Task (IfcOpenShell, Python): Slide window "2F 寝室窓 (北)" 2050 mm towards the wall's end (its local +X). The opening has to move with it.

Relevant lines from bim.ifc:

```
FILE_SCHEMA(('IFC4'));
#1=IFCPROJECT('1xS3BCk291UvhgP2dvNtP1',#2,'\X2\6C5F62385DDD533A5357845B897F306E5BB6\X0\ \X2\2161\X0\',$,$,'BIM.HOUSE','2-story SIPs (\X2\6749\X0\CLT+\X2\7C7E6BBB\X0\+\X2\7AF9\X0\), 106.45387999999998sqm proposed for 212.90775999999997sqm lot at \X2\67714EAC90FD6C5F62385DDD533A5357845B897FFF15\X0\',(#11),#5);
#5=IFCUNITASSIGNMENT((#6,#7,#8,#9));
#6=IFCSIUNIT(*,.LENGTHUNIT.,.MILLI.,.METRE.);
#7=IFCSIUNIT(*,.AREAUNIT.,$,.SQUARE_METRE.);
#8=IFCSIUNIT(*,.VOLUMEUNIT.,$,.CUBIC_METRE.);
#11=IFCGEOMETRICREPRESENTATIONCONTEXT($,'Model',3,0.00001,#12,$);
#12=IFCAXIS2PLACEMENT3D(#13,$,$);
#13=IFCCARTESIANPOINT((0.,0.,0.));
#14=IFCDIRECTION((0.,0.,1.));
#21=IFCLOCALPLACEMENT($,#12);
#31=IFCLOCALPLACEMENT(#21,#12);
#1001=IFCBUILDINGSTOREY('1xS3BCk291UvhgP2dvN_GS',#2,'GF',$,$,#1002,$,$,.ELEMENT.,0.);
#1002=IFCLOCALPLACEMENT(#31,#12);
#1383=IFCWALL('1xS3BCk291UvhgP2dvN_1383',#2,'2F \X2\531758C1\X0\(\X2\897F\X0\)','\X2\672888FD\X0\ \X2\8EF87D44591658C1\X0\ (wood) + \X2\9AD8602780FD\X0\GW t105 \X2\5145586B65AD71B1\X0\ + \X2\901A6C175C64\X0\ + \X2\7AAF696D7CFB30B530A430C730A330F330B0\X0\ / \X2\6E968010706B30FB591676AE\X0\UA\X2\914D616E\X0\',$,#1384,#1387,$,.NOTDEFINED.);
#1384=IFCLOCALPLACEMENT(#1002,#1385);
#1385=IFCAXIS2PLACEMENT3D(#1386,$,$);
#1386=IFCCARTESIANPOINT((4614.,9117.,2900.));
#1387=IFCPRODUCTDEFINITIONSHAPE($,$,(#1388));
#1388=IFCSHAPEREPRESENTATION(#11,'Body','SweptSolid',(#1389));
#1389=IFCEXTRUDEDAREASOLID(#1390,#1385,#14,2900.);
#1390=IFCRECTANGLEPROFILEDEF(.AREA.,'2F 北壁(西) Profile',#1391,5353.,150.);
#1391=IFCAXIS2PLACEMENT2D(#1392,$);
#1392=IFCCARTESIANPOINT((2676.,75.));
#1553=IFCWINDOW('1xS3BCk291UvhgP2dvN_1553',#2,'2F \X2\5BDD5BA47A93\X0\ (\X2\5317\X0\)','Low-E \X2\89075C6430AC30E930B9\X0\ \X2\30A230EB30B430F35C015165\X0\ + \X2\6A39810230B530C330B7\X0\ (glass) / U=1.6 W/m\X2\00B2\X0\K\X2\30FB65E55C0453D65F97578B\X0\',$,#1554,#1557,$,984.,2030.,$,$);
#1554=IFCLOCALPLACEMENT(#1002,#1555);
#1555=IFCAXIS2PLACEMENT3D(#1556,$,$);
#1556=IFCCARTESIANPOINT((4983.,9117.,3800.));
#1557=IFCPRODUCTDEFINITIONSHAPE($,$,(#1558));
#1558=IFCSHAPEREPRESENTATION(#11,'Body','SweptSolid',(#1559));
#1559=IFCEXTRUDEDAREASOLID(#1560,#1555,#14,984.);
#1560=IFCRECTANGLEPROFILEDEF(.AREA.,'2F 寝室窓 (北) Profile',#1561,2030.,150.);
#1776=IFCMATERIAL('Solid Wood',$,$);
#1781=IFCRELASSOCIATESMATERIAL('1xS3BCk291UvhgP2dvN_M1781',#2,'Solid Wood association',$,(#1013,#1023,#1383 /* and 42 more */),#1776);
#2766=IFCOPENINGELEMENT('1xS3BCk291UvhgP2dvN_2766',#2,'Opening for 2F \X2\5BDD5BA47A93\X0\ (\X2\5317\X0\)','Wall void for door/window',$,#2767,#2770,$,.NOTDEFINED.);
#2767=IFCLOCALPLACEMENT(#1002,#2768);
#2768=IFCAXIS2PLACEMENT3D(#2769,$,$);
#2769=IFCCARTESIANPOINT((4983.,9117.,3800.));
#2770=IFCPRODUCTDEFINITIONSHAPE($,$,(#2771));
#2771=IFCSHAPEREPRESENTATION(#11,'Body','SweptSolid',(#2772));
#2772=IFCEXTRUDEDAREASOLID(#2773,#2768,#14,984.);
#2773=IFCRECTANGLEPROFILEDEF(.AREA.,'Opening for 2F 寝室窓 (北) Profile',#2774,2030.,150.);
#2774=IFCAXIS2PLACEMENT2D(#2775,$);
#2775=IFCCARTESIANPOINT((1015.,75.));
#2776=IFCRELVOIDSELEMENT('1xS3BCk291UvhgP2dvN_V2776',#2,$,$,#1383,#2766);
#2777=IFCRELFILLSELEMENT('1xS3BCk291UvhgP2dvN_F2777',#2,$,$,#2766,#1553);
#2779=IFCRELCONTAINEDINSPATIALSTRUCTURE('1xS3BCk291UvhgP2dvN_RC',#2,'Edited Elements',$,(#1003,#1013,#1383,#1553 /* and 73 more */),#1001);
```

```python
import ifcopenshell
import ifcopenshell.api.geometry
import ifcopenshell.util.placement
import ifcopenshell.util.unit

model = ifcopenshell.open("bim.ifc")
unit_scale = ifcopenshell.util.unit.calculate_unit_scale(model)

window = model.by_guid("1xS3BCk291UvhgP2dvN_1553")
opening = window.FillsVoids[0].RelatingOpeningElement
wall = opening.VoidsElements[0].RelatingBuildingElement

wall_matrix = ifcopenshell.util.placement.get_local_placement(wall.ObjectPlacement)
shift = wall_matrix[:3, 0] * 2.05 / unit_scale
before = ifcopenshell.util.placement.get_local_placement(window.ObjectPlacement)[:3, 3].copy()

# The window is not placed relative to its opening, so move both.
for product in (opening, window):
    matrix = ifcopenshell.util.placement.get_local_placement(product.ObjectPlacement)
    matrix[:3, 3] += shift
    ifcopenshell.api.geometry.edit_object_placement(model, product=product, matrix=matrix, is_si=False)

after = ifcopenshell.util.placement.get_local_placement(window.ObjectPlacement)[:3, 3]
print("window moved by", (after - before).round(3) + 0.0)

model.write("bim_edited.ifc")
```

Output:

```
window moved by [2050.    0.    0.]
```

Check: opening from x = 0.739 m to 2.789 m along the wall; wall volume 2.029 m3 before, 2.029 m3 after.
